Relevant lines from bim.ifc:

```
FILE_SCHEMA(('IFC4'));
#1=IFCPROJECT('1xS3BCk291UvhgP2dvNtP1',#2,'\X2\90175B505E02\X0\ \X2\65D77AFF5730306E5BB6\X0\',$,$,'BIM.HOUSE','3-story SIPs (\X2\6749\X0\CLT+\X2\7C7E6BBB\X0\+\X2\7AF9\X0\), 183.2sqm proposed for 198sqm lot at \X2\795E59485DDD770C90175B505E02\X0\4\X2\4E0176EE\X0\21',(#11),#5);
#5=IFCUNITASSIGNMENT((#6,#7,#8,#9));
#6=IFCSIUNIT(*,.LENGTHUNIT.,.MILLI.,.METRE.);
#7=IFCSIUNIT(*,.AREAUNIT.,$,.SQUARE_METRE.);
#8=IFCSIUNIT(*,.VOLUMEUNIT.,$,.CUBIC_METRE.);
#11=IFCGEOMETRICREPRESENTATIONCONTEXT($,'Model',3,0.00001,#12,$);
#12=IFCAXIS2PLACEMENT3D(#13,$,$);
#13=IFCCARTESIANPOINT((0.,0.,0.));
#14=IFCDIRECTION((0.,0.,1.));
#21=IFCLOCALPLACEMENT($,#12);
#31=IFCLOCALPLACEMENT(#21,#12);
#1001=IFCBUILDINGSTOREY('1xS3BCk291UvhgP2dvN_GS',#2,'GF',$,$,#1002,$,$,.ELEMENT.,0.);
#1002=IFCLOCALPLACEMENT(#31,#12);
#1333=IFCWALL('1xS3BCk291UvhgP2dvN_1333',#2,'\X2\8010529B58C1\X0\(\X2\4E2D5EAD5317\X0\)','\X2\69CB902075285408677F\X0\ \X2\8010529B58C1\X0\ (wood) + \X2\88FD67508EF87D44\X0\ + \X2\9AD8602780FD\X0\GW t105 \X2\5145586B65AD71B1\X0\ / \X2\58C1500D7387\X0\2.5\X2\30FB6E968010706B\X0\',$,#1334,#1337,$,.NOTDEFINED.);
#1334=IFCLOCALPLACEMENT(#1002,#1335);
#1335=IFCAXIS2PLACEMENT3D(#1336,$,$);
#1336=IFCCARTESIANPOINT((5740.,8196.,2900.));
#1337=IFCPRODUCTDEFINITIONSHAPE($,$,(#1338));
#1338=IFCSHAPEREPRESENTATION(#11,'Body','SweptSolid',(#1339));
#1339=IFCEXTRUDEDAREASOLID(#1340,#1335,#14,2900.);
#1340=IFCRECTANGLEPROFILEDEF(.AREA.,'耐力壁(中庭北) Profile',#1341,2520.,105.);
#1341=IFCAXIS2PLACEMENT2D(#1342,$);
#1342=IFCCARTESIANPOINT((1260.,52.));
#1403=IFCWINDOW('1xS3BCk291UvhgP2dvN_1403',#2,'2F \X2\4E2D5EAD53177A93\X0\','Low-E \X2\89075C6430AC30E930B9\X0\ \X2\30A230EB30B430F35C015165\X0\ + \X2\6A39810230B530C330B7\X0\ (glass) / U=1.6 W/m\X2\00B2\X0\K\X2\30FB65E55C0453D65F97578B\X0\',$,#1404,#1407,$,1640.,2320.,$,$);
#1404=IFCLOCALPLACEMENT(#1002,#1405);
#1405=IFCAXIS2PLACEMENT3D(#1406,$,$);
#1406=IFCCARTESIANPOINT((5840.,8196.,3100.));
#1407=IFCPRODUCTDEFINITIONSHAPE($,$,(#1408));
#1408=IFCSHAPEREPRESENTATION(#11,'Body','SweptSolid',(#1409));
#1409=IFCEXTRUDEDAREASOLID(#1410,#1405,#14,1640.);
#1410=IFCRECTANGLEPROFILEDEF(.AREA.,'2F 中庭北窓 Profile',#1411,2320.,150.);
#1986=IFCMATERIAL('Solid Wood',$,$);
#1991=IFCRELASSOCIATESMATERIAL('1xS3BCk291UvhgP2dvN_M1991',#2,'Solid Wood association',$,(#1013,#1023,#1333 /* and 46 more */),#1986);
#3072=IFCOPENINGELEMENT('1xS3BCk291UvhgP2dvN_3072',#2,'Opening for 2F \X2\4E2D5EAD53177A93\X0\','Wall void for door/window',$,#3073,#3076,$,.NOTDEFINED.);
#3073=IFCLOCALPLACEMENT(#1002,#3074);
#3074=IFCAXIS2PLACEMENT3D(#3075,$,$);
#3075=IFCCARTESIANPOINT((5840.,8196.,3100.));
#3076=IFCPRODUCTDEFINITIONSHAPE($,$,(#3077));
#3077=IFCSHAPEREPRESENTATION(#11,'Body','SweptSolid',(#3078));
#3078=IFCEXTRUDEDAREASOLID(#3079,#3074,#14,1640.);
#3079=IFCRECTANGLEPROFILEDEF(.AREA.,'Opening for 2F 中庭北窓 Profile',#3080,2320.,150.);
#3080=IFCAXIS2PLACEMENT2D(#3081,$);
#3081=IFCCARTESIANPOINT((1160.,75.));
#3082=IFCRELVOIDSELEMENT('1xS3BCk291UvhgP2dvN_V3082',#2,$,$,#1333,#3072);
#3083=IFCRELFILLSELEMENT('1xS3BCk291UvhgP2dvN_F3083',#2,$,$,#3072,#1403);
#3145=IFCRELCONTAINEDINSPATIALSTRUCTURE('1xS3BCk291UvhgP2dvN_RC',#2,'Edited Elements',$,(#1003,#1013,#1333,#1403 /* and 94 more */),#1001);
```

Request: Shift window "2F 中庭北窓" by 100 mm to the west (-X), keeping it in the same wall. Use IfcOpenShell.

```python
import ifcopenshell
import ifcopenshell.api.geometry
import ifcopenshell.util.placement
import ifcopenshell.util.unit

model = ifcopenshell.open("bim.ifc")
unit_scale = ifcopenshell.util.unit.calculate_unit_scale(model)

window = model.by_guid("1xS3BCk291UvhgP2dvN_1403")
opening = window.FillsVoids[0].RelatingOpeningElement
wall = opening.VoidsElements[0].RelatingBuildingElement

wall_matrix = ifcopenshell.util.placement.get_local_placement(wall.ObjectPlacement)
shift = wall_matrix[:3, 0] * -0.1 / unit_scale
before = ifcopenshell.util.placement.get_local_placement(window.ObjectPlacement)[:3, 3].copy()

# The window is not placed relative to its opening, so move both.
for product in (opening, window):
    matrix = ifcopenshell.util.placement.get_local_placement(product.ObjectPlacement)
    matrix[:3, 3] += shift
    ifcopenshell.api.geometry.edit_object_placement(model, product=product, matrix=matrix, is_si=False)

after = ifcopenshell.util.placement.get_local_placement(window.ObjectPlacement)[:3, 3]
print("window moved by", (after - before).round(3) + 0.0)

model.write("bim_rev.ifc")
```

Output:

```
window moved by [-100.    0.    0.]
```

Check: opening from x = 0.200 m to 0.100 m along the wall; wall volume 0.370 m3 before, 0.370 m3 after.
